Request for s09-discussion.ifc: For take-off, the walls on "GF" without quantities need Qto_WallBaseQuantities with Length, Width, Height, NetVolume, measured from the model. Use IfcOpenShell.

First a look at what the model holds.

```python
import ifcopenshell
import ifcopenshell.util.element
import ifcopenshell.util.unit

model = ifcopenshell.open("s09-discussion.ifc")
print(model.schema)
for unit_type in ("LENGTHUNIT", "AREAUNIT", "VOLUMEUNIT"):
    print(unit_type, ifcopenshell.util.unit.calculate_unit_scale(model, unit_type))
storey = next(s for s in model.by_type("IfcBuildingStorey") if s.Name == "GF")
walls = [e for e in ifcopenshell.util.element.get_decomposition(storey) if e.is_a("IfcWall")]
for e in sorted(walls, key=lambda e: e.id()):
    print(e.id(), e.is_a(), e.Name, list(ifcopenshell.util.element.get_psets(e, qtos_only=True)), sep=" | ")
```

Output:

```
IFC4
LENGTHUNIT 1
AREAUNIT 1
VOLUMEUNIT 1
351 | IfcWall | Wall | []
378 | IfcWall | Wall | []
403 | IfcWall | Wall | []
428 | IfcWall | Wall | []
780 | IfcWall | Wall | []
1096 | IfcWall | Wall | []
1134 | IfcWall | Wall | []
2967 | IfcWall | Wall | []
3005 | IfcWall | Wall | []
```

```python
import ifcopenshell
import ifcopenshell.api.pset
import ifcopenshell.geom
import ifcopenshell.util.element
import ifcopenshell.util.shape
import ifcopenshell.util.unit

model = ifcopenshell.open("s09-discussion.ifc")
unit_scale = ifcopenshell.util.unit.calculate_unit_scale(model)
volume_scale = ifcopenshell.util.unit.calculate_unit_scale(model, "VOLUMEUNIT")
settings = ifcopenshell.geom.settings()

storey = next(s for s in model.by_type("IfcBuildingStorey") if s.Name == "GF")
walls = [e for e in ifcopenshell.util.element.get_decomposition(storey) if e.is_a("IfcWall")]

for e in sorted(walls, key=lambda e: e.id()):
    if ifcopenshell.util.element.get_psets(e, qtos_only=True, should_inherit=False):
        continue
    # Geometry comes back in metres, in the element's own axes.
    shape = ifcopenshell.geom.create_shape(settings, e)
    values = {
        "Length": ifcopenshell.util.shape.get_x(shape.geometry) / unit_scale,
        "Width": ifcopenshell.util.shape.get_y(shape.geometry) / unit_scale,
        "Height": ifcopenshell.util.shape.get_z(shape.geometry) / unit_scale,
        "NetVolume": ifcopenshell.util.shape.get_volume(shape.geometry) / volume_scale,
    }
    qto = ifcopenshell.api.pset.add_qto(model, product=e, name="Qto_WallBaseQuantities")
    ifcopenshell.api.pset.edit_qto(model, qto=qto, properties=values)
    print(e.id(), {k: round(v, 3) for k, v in values.items()})

model.write("s09-discussion_rev.ifc")
```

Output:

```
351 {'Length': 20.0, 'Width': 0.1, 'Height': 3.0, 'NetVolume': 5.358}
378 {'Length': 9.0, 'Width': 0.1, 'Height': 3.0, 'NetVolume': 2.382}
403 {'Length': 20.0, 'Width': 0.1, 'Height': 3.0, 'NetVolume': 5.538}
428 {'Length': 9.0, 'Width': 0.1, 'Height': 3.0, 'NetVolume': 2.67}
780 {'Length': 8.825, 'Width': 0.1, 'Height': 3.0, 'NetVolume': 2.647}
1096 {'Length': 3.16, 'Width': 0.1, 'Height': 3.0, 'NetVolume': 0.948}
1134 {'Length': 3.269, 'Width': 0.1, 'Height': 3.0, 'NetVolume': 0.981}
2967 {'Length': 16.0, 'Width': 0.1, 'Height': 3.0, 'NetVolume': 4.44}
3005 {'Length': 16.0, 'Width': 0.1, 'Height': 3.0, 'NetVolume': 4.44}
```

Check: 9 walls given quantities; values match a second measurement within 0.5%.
